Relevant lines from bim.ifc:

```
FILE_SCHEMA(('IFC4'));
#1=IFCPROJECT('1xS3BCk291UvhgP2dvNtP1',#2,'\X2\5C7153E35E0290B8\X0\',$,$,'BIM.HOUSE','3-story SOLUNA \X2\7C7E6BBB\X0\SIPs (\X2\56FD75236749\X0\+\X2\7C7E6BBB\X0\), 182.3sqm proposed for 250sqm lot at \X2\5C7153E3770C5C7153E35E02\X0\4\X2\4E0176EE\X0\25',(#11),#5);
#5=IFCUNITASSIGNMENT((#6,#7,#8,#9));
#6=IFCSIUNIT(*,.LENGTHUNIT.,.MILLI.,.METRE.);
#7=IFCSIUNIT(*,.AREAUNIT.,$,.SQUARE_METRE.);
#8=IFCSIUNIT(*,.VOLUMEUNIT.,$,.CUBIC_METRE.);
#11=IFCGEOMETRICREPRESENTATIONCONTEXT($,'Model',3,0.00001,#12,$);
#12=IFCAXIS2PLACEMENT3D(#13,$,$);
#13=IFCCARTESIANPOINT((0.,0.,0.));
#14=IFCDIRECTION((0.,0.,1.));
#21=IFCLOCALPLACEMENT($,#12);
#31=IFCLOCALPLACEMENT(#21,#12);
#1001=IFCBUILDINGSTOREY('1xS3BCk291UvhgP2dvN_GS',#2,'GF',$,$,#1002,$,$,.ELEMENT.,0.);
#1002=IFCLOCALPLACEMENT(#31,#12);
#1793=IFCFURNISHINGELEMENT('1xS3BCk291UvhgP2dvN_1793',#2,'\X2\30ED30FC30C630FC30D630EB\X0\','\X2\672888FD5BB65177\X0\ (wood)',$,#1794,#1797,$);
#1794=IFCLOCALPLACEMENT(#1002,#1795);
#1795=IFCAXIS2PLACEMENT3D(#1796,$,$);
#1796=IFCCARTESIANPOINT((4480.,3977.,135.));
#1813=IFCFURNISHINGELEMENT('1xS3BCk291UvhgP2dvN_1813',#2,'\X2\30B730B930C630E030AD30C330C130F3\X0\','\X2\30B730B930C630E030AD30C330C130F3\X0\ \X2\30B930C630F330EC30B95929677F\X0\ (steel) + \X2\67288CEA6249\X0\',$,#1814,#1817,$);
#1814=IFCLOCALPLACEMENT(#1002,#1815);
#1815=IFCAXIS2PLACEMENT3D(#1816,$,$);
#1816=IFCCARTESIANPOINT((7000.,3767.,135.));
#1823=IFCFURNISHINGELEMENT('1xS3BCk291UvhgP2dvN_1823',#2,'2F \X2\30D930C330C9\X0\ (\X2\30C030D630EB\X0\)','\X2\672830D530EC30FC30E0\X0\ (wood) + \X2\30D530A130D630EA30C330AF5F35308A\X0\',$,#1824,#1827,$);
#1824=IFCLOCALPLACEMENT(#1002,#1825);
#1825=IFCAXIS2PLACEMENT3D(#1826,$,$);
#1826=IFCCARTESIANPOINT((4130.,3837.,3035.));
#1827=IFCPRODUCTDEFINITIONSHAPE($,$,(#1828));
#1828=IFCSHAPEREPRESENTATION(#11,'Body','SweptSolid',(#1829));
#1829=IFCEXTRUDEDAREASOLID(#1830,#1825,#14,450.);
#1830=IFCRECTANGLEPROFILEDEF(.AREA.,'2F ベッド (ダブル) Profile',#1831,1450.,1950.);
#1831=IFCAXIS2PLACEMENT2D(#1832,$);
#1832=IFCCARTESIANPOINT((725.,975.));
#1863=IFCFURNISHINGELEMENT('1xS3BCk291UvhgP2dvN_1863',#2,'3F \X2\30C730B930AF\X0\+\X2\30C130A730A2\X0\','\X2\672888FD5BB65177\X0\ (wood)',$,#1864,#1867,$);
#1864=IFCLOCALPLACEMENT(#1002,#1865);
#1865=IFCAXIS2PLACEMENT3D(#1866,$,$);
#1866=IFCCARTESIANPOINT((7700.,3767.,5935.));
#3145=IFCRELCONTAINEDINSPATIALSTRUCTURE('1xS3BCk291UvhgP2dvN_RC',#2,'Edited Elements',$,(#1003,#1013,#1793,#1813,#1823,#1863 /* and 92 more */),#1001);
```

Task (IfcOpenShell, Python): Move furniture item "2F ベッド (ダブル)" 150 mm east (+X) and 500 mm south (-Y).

```python
import ifcopenshell
import ifcopenshell.api.geometry
import ifcopenshell.util.placement
import ifcopenshell.util.unit

model = ifcopenshell.open("bim.ifc")
unit_scale = ifcopenshell.util.unit.calculate_unit_scale(model)

item = model.by_guid("1xS3BCk291UvhgP2dvN_1823")
matrix = ifcopenshell.util.placement.get_local_placement(item.ObjectPlacement)
matrix[0, 3] += 0.15 / unit_scale
matrix[1, 3] -= 0.5 / unit_scale
ifcopenshell.api.geometry.edit_object_placement(model, product=item, matrix=matrix, is_si=False)

print(ifcopenshell.util.placement.get_local_placement(item.ObjectPlacement).round(3) + 0.0)

model.write("bim-out.ifc")
```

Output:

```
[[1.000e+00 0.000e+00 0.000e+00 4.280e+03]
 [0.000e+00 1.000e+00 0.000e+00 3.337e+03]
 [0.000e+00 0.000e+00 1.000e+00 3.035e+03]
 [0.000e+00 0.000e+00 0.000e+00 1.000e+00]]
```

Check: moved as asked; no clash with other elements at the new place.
